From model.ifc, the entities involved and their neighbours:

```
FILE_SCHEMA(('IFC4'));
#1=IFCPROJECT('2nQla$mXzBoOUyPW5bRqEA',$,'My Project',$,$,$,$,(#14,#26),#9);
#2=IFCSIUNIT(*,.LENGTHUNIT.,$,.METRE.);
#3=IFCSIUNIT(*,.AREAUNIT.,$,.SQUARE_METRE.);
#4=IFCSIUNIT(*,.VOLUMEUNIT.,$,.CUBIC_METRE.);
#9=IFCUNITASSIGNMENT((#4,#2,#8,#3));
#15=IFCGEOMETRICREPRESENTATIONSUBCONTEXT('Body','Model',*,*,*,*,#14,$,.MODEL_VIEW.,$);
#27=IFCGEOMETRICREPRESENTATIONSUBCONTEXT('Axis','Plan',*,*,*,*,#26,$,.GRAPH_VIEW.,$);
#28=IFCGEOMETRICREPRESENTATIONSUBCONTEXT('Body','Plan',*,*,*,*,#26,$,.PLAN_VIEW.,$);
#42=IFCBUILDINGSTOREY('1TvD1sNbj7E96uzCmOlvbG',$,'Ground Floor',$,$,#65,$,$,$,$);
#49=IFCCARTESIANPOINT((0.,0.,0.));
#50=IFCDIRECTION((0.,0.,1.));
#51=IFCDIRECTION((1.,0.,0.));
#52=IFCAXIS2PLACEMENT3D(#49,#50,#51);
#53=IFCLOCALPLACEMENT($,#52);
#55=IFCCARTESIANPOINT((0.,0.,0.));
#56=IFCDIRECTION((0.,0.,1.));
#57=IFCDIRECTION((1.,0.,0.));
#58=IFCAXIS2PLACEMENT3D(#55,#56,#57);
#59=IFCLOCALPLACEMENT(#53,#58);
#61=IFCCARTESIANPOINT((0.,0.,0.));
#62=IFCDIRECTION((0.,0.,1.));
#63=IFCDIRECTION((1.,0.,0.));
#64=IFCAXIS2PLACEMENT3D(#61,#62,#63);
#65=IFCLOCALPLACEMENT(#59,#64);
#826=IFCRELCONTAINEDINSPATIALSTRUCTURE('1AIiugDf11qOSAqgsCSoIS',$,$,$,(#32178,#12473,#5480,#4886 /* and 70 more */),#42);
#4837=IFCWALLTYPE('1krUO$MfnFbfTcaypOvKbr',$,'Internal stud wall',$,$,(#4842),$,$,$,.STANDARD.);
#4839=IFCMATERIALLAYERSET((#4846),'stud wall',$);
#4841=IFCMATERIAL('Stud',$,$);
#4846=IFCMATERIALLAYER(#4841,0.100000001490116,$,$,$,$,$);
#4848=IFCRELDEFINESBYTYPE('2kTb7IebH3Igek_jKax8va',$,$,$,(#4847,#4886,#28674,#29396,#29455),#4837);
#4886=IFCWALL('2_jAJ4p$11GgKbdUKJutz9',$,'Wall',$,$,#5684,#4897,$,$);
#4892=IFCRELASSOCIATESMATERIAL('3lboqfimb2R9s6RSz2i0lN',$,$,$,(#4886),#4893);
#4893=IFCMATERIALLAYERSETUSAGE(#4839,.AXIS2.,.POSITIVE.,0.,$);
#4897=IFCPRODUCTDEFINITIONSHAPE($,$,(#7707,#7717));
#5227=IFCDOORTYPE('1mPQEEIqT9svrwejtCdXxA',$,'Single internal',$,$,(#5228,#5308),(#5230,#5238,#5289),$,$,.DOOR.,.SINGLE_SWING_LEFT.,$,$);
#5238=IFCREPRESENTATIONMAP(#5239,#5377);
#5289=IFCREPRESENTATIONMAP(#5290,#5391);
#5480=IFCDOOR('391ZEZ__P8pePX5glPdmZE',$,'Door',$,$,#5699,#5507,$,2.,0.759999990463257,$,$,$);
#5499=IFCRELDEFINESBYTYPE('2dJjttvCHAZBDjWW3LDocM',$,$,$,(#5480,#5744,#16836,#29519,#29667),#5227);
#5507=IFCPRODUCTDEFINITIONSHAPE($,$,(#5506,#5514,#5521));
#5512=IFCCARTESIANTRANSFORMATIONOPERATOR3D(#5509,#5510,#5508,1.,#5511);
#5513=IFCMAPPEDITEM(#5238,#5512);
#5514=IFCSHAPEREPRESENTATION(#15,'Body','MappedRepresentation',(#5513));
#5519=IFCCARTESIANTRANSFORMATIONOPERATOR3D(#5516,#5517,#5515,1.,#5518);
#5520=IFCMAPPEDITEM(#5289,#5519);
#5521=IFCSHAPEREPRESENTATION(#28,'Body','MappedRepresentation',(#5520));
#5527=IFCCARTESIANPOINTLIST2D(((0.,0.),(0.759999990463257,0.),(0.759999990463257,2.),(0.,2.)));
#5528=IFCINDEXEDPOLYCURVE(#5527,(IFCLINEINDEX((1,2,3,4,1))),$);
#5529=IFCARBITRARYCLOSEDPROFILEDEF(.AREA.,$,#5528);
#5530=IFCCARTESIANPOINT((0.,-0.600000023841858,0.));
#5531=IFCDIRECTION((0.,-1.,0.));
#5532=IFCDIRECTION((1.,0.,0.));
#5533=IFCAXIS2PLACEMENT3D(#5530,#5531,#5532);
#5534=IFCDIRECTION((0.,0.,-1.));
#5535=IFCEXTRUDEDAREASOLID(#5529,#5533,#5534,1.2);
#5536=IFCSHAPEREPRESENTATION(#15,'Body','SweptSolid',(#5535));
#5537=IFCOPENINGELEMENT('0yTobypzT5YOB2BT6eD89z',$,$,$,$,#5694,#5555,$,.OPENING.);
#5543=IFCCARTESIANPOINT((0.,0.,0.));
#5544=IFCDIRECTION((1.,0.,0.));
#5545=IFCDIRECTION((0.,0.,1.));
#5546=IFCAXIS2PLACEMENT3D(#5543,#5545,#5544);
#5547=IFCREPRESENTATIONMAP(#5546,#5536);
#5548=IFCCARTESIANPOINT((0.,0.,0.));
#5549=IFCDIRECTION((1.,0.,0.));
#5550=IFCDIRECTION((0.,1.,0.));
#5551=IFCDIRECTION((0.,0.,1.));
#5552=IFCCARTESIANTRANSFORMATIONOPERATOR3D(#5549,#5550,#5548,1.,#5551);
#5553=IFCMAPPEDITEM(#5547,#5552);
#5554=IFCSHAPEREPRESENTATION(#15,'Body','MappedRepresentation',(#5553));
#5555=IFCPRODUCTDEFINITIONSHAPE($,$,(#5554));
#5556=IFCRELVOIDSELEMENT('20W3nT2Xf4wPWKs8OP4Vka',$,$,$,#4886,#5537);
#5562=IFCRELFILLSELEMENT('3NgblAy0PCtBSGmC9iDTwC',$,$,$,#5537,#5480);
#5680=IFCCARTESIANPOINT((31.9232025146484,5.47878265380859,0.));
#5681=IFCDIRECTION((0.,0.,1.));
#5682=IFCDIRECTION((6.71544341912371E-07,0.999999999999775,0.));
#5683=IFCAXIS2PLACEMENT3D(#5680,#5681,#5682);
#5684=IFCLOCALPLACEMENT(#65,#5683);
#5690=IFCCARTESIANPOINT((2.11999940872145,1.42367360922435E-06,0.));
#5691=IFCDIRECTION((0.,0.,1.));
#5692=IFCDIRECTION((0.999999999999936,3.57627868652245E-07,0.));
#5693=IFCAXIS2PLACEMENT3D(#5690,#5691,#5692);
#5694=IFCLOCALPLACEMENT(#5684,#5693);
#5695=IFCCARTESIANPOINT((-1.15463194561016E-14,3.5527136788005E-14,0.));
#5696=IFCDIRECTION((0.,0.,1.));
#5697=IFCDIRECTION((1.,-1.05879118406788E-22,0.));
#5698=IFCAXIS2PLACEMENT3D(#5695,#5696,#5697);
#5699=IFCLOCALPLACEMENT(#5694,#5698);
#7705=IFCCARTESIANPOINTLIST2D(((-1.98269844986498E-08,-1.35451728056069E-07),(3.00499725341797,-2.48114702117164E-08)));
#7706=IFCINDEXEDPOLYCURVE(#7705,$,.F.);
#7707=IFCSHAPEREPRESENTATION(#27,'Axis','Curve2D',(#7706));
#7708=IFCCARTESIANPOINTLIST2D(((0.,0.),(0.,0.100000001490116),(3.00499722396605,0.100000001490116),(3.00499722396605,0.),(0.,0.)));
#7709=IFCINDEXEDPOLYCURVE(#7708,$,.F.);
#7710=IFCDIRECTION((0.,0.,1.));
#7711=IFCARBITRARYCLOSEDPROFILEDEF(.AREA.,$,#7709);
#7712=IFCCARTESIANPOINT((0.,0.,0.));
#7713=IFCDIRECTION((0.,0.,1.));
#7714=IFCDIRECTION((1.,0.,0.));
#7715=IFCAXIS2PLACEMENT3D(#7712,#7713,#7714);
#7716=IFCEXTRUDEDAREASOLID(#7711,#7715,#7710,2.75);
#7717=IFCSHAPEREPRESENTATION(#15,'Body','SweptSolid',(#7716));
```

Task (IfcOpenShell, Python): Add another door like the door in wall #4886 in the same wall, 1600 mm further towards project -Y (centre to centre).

```python
import ifcopenshell
import ifcopenshell.api.feature
import ifcopenshell.api.geometry
import ifcopenshell.api.root
import ifcopenshell.geom
import ifcopenshell.util.element
import ifcopenshell.util.placement
import ifcopenshell.util.shape

model = ifcopenshell.open("model.ifc")
settings = ifcopenshell.geom.settings()


def volume(element):
    """Net volume in cubic metres, openings subtracted."""
    shape = ifcopenshell.geom.create_shape(settings, element)
    return ifcopenshell.util.shape.get_volume(shape.geometry)


door = model.by_guid("391ZEZ__P8pePX5glPdmZE")
opening = door.FillsVoids[0].RelatingOpeningElement
wall = opening.VoidsElements[0].RelatingBuildingElement
before = volume(wall)
shift = ifcopenshell.util.placement.get_local_placement(wall.ObjectPlacement)[:3, 0] * -1.6

# copy_class copies the void relationship, type, container and properties, but no geometry.
new_opening = ifcopenshell.api.root.copy_class(model, product=opening)
new_opening.Representation = ifcopenshell.util.element.copy_deep(
    model, opening.Representation, exclude=["IfcGeometricRepresentationContext", "IfcRepresentationMap"]
)
new_door = ifcopenshell.api.root.copy_class(model, product=door)
new_door.Representation = ifcopenshell.util.element.copy_deep(
    model, door.Representation, exclude=["IfcGeometricRepresentationContext", "IfcRepresentationMap"]
)
ifcopenshell.api.feature.add_filling(model, opening=new_opening, element=new_door)

for old, new in ((opening, new_opening), (door, new_door)):
    matrix = ifcopenshell.util.placement.get_local_placement(old.ObjectPlacement)
    matrix[:3, 3] += shift
    ifcopenshell.api.geometry.edit_object_placement(model, product=new, matrix=matrix, is_si=False)

after = volume(wall)

print(f"wall volume {before:.3f} -> {after:.3f} m3")

model.write("model_edited.ifc")
```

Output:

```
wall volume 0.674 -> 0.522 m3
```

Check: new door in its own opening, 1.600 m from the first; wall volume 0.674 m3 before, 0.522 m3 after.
